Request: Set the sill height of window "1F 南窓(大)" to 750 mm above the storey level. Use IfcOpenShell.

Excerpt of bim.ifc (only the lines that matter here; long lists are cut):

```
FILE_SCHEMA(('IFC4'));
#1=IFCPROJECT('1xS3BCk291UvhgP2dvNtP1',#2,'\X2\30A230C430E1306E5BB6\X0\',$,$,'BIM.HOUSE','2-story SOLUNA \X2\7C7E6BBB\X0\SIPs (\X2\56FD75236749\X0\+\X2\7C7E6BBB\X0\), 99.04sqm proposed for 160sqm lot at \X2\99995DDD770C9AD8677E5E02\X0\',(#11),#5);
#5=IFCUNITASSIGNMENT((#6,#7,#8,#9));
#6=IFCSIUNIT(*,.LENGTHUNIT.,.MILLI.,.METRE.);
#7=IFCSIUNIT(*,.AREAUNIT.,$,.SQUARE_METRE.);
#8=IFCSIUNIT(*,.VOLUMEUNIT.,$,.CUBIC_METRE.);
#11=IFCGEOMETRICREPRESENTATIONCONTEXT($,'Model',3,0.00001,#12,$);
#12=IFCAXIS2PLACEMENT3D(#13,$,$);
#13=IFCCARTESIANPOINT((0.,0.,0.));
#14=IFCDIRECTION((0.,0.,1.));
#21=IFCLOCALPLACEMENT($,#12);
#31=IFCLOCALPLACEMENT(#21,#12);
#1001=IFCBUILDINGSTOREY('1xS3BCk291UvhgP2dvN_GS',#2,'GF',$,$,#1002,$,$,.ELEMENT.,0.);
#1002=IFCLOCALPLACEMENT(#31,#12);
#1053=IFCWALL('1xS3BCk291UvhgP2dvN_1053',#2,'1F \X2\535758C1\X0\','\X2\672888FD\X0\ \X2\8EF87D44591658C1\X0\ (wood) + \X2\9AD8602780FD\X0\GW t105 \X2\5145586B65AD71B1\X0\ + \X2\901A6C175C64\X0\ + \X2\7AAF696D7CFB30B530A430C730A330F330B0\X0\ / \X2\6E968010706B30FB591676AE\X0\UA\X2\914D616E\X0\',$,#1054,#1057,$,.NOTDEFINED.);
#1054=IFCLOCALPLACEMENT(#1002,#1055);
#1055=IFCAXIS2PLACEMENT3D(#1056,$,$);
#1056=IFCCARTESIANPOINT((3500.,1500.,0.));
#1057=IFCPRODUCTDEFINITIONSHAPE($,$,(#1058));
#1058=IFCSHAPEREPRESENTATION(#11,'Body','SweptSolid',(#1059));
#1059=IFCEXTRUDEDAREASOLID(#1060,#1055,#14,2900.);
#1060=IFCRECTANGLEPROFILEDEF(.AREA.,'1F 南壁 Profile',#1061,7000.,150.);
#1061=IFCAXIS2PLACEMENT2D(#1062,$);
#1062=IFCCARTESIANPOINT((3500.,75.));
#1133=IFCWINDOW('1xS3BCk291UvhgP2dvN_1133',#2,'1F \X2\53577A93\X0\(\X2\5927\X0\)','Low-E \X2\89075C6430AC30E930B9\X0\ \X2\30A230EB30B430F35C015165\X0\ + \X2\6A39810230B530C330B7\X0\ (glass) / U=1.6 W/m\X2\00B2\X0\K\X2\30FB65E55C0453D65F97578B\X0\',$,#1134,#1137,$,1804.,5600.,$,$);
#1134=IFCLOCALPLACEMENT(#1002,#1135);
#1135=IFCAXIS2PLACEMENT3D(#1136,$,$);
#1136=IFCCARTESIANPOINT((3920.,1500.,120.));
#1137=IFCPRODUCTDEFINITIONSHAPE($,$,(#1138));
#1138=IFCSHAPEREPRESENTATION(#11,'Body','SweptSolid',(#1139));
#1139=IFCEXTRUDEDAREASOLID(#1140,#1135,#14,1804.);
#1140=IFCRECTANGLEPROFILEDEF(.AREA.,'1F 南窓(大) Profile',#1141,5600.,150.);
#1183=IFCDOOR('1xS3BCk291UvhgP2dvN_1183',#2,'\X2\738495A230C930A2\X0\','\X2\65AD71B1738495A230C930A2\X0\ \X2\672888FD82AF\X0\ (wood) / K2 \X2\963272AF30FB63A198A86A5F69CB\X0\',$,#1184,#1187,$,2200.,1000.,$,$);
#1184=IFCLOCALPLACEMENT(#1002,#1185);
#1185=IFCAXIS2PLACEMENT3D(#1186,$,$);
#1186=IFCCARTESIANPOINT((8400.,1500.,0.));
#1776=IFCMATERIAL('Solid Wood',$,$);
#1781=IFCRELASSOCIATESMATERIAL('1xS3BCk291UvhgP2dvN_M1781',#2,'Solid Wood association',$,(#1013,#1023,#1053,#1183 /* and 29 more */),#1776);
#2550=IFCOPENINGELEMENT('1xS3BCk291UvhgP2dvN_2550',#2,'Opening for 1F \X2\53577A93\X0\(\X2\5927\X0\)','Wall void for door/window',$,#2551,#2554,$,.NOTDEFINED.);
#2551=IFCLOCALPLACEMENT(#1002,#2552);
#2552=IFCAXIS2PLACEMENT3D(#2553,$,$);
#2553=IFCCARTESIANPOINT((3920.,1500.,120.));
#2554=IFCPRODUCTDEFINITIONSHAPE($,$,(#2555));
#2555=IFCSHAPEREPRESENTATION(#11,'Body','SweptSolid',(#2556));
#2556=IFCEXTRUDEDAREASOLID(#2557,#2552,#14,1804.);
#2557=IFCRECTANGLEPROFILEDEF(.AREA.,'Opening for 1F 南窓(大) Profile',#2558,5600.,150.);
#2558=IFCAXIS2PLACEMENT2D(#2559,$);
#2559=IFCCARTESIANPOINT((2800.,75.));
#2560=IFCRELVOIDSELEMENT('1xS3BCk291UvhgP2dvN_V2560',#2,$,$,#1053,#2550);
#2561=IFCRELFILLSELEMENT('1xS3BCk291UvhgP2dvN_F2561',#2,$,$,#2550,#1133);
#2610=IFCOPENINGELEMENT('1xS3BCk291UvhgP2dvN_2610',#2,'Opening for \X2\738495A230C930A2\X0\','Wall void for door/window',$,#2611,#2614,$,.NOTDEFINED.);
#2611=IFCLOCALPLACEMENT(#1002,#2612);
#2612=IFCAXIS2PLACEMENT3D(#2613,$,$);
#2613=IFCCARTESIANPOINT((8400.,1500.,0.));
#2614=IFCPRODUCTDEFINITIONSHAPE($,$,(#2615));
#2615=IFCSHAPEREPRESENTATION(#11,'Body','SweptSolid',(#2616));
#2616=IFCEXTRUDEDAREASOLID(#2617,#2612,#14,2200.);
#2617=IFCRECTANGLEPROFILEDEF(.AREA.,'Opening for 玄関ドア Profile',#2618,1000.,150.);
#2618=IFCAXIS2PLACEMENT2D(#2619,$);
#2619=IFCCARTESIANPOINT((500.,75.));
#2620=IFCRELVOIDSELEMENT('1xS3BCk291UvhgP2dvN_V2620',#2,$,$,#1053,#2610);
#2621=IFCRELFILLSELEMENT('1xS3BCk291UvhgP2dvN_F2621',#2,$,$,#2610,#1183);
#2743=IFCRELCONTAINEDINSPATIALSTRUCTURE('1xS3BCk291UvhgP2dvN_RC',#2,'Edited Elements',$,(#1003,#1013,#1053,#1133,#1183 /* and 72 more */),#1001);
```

```python
import numpy as np
import ifcopenshell
import ifcopenshell.api.geometry
import ifcopenshell.geom
import ifcopenshell.util.element
import ifcopenshell.util.placement
import ifcopenshell.util.shape
import ifcopenshell.util.unit

model = ifcopenshell.open("bim.ifc")
unit_scale = ifcopenshell.util.unit.calculate_unit_scale(model)

window = model.by_guid("1xS3BCk291UvhgP2dvN_1133")
opening = window.FillsVoids[0].RelatingOpeningElement
storey = ifcopenshell.util.element.get_container(window, ifc_class="IfcBuildingStorey")
level = ifcopenshell.util.placement.get_local_placement(storey.ObjectPlacement)[2, 3]

# The opening's origin need not be at the sill, so measure its lowest point.
shape = ifcopenshell.geom.create_shape(ifcopenshell.geom.settings(), opening)
bottom = ifcopenshell.util.shape.get_shape_bottom_elevation(shape, shape.geometry) / unit_scale
dz = level + 0.75 / unit_scale - bottom

shift = np.array([0.0, 0.0, dz])
# The window is not placed relative to its opening, so move both.
for product in (opening, window):
    matrix = ifcopenshell.util.placement.get_local_placement(product.ObjectPlacement)
    matrix[:3, 3] += shift
    ifcopenshell.api.geometry.edit_object_placement(model, product=product, matrix=matrix, is_si=False)

print(f"moved by {dz * unit_scale:+.3f} m")

model.write("bim-out.ifc")
```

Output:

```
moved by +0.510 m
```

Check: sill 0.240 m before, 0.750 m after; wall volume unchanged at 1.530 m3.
